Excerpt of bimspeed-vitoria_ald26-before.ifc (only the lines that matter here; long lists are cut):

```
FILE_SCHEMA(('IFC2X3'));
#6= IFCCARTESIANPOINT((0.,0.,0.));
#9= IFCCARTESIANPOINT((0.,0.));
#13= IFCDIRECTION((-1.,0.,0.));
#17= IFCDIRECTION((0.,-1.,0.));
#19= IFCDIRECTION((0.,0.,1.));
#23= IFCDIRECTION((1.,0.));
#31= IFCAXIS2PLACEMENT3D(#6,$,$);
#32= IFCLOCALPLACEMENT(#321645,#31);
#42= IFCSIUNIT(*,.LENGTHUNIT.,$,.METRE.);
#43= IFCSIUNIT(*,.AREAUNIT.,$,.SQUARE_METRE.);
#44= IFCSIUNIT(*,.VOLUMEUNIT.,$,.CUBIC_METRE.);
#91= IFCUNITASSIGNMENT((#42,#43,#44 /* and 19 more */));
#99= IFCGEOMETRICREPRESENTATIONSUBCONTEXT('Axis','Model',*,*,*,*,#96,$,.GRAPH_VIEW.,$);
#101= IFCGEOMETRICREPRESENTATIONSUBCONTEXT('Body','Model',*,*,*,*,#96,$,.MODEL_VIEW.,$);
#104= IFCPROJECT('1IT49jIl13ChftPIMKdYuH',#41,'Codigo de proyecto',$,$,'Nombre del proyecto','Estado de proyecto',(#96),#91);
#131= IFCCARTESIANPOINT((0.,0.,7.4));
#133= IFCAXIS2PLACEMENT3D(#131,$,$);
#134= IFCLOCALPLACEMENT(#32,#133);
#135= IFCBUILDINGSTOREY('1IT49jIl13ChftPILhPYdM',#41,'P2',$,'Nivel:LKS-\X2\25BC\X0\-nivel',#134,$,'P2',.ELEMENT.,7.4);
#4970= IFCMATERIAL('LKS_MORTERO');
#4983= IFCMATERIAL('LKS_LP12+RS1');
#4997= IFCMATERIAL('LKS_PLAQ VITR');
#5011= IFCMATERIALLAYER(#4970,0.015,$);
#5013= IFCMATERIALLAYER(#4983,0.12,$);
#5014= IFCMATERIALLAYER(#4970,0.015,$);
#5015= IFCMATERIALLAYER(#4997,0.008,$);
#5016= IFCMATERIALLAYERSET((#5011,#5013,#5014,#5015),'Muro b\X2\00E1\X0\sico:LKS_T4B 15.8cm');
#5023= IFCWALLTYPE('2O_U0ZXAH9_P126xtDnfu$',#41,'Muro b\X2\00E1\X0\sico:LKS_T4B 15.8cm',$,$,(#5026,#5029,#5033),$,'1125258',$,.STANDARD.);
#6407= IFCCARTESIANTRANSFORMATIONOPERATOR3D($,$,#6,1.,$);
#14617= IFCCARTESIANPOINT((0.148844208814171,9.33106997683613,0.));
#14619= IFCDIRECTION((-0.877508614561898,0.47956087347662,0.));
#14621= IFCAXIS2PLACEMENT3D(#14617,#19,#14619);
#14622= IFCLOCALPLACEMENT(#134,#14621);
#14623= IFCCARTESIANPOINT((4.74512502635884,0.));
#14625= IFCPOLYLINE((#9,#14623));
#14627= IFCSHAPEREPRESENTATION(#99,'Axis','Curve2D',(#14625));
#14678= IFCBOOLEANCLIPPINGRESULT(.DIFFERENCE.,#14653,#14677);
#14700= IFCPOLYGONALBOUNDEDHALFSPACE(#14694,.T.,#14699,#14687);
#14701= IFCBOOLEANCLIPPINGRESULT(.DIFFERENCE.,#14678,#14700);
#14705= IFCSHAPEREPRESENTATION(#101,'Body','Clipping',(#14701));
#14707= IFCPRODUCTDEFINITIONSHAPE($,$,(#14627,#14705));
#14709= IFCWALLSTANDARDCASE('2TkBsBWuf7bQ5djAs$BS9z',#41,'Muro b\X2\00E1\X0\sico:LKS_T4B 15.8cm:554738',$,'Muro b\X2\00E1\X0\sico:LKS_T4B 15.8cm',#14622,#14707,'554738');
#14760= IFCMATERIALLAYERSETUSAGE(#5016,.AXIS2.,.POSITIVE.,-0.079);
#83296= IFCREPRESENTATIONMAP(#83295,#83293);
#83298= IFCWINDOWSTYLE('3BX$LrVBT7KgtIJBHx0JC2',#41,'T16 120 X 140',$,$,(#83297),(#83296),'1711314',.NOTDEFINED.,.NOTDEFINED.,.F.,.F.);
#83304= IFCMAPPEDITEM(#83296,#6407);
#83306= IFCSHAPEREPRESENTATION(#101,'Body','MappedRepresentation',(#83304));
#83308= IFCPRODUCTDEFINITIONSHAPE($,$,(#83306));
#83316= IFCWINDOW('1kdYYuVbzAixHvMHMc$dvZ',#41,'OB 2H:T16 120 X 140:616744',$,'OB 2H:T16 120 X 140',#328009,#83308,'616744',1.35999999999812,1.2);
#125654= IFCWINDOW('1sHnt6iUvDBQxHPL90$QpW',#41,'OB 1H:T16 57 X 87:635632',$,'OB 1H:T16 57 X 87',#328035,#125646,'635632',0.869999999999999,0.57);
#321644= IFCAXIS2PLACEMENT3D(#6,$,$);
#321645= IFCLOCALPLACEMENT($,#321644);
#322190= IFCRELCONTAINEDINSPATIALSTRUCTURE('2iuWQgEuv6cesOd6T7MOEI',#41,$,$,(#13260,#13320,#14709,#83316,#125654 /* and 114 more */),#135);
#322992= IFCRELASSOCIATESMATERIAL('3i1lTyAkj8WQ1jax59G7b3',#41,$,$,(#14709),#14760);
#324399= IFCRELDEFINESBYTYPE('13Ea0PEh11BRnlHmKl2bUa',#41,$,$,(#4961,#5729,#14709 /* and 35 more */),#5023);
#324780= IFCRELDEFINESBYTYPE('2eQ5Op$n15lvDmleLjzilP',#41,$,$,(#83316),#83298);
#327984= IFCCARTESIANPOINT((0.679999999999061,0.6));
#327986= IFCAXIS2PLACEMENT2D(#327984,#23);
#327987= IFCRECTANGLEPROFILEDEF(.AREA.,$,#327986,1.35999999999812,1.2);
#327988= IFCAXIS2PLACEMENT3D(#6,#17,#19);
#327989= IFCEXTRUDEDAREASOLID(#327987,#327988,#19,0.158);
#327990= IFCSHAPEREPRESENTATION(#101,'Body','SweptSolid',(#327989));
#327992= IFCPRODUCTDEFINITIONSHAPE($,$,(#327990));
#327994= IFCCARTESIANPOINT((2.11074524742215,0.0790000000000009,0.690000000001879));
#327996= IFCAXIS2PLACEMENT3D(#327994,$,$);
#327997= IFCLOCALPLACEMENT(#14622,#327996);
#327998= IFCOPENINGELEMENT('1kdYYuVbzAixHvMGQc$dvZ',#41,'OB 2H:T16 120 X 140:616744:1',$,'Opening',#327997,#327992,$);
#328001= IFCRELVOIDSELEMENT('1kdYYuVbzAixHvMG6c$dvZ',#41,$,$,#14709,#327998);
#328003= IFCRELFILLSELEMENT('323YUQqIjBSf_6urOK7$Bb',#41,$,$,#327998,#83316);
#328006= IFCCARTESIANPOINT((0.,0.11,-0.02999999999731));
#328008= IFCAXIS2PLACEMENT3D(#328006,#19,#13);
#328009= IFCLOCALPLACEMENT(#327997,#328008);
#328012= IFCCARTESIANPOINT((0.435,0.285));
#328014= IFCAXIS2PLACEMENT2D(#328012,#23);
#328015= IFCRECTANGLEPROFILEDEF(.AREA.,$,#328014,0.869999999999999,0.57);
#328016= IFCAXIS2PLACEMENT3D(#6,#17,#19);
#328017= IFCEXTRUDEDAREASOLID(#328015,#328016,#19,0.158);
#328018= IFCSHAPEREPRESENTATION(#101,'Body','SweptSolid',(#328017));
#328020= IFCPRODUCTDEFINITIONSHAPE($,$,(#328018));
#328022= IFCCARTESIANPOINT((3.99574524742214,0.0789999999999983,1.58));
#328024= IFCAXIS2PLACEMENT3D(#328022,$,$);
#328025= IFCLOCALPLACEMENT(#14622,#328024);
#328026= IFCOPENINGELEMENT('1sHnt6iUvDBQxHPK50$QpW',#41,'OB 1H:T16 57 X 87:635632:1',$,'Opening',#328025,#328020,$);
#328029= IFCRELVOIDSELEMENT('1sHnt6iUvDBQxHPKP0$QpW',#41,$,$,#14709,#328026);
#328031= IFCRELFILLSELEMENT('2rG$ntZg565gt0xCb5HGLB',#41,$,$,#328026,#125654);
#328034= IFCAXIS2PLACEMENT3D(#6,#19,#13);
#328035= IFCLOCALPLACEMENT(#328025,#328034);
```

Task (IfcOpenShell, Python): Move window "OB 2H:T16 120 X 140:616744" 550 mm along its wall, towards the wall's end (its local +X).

```python
import ifcopenshell
import ifcopenshell.api.geometry
import ifcopenshell.util.placement
import ifcopenshell.util.unit

model = ifcopenshell.open("bimspeed-vitoria_ald26-before.ifc")
unit_scale = ifcopenshell.util.unit.calculate_unit_scale(model)

window = model.by_guid("1kdYYuVbzAixHvMHMc$dvZ")
opening = window.FillsVoids[0].RelatingOpeningElement
wall = opening.VoidsElements[0].RelatingBuildingElement

wall_matrix = ifcopenshell.util.placement.get_local_placement(wall.ObjectPlacement)
shift = wall_matrix[:3, 0] * 0.55 / unit_scale
before = ifcopenshell.util.placement.get_local_placement(window.ObjectPlacement)[:3, 3].copy()

# The window is placed relative to its opening, so it follows when the opening moves.
matrix = ifcopenshell.util.placement.get_local_placement(opening.ObjectPlacement)
matrix[:3, 3] += shift
ifcopenshell.api.geometry.edit_object_placement(
    model, product=opening, matrix=matrix, is_si=False, should_transform_children=True
)

after = ifcopenshell.util.placement.get_local_placement(window.ObjectPlacement)[:3, 3]
print("window moved by", (after - before).round(3) + 0.0)

model.write("bimspeed-vitoria_ald26-before_rev.ifc")
```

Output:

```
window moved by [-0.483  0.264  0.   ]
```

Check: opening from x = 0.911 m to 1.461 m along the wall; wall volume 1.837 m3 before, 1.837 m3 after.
